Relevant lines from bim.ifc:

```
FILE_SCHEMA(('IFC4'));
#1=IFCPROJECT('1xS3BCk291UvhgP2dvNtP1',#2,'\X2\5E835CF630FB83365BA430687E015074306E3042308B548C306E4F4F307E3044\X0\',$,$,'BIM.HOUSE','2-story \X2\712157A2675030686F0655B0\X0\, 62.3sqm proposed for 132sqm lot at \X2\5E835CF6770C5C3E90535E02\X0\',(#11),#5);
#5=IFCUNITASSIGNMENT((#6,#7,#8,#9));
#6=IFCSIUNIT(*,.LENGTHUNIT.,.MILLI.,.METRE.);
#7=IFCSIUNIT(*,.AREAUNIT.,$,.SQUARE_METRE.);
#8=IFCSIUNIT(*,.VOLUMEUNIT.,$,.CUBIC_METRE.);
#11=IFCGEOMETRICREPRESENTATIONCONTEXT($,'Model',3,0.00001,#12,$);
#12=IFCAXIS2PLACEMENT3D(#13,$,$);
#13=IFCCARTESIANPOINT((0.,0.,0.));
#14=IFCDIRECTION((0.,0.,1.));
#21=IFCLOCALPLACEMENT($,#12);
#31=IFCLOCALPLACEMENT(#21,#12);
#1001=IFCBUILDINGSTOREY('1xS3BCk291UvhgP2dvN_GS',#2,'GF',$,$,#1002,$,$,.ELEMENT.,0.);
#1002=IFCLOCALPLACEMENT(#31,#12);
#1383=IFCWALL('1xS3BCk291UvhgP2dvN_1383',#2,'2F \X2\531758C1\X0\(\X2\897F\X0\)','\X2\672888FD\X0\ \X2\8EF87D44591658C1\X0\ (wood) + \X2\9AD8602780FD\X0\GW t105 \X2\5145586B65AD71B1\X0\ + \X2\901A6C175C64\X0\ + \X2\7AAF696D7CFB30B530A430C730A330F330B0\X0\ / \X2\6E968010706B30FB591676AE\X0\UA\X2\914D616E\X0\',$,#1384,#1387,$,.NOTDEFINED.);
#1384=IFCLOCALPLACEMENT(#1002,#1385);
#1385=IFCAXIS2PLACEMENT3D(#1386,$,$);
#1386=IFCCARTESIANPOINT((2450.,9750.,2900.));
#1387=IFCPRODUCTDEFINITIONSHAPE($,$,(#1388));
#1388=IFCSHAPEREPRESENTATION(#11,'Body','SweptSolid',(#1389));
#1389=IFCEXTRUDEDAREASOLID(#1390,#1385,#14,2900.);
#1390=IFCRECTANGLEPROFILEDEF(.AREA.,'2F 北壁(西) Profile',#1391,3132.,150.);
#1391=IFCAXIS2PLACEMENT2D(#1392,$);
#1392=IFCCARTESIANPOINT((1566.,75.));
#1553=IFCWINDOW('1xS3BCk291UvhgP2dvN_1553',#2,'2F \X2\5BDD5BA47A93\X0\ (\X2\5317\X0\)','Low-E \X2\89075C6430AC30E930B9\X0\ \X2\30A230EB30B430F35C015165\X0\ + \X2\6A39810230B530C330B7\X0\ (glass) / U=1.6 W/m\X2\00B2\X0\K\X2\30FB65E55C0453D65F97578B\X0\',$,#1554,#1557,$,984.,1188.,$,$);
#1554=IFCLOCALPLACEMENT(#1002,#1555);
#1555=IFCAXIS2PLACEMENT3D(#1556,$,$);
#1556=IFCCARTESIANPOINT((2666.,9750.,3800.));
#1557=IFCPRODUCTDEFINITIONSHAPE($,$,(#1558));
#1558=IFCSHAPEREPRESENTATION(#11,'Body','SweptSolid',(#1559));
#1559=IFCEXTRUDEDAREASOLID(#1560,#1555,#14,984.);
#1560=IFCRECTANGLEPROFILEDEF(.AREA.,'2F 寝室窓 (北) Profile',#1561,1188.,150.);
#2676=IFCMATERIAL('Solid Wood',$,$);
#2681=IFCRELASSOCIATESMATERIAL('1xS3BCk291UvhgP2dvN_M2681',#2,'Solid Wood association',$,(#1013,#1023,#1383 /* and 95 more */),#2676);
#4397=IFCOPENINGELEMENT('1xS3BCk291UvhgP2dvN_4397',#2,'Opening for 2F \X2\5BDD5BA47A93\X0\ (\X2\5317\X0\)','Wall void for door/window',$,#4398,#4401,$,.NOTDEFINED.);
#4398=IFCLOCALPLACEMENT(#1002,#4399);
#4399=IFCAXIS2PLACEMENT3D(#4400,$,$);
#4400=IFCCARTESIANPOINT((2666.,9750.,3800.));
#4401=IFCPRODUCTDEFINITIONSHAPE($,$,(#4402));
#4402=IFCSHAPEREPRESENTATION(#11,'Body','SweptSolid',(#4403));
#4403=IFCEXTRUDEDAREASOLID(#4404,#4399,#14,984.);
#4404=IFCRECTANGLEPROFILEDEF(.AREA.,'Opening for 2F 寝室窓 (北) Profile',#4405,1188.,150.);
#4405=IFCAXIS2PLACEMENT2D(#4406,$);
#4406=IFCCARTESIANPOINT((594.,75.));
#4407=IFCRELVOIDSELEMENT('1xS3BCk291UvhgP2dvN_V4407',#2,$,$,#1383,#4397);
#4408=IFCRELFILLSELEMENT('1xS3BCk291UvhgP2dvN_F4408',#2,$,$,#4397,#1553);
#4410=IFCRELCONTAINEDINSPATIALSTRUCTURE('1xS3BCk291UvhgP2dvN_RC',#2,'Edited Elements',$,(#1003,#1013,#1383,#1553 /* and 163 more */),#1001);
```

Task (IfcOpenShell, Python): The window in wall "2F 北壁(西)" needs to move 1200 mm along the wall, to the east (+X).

```python
import ifcopenshell
import ifcopenshell.api.geometry
import ifcopenshell.util.placement
import ifcopenshell.util.unit

model = ifcopenshell.open("bim.ifc")
unit_scale = ifcopenshell.util.unit.calculate_unit_scale(model)

window = model.by_id(1553)
opening = window.FillsVoids[0].RelatingOpeningElement
wall = opening.VoidsElements[0].RelatingBuildingElement

wall_matrix = ifcopenshell.util.placement.get_local_placement(wall.ObjectPlacement)
shift = wall_matrix[:3, 0] * 1.2 / unit_scale
before = ifcopenshell.util.placement.get_local_placement(window.ObjectPlacement)[:3, 3].copy()

# The window is not placed relative to its opening, so move both.
for product in (opening, window):
    matrix = ifcopenshell.util.placement.get_local_placement(product.ObjectPlacement)
    matrix[:3, 3] += shift
    ifcopenshell.api.geometry.edit_object_placement(model, product=product, matrix=matrix, is_si=False)

after = ifcopenshell.util.placement.get_local_placement(window.ObjectPlacement)[:3, 3]
print("window moved by", (after - before).round(3) + 0.0)

model.write("bim_updated.ifc")
```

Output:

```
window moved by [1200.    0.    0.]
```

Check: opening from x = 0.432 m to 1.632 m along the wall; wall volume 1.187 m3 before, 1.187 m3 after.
